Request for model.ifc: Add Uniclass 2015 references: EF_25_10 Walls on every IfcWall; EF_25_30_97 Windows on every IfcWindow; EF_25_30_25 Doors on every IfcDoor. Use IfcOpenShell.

First a look at what the model holds.

```python
import ifcopenshell

model = ifcopenshell.open("model.ifc")
print(model.schema)
print("classifications:", [c.Name for c in model.by_type("IfcClassification")])
for ifc_class in ("IfcDoor", "IfcRoof", "IfcStair", "IfcWall", "IfcWindow"):
    print(ifc_class, len(model.by_type(ifc_class)))
```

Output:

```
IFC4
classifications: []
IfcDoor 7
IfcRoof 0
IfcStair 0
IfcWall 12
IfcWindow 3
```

```python
import ifcopenshell
import ifcopenshell.api.classification

model = ifcopenshell.open("model.ifc")

system = ifcopenshell.api.classification.add_classification(model, classification="Uniclass 2015")

codes = {
    "IfcWall": ("EF_25_10", "Walls"),
    "IfcWindow": ("EF_25_30_97", "Windows"),
    "IfcDoor": ("EF_25_30_25", "Doors"),
}
for ifc_class, (code, name) in codes.items():
    products = model.by_type(ifc_class)
    ifcopenshell.api.classification.add_reference(
        model, products=products, classification=system, identification=code, name=name
    )
    print(code, len(products))

model.write("model_rev.ifc")
```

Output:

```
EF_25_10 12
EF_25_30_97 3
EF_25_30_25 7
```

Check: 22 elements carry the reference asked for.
